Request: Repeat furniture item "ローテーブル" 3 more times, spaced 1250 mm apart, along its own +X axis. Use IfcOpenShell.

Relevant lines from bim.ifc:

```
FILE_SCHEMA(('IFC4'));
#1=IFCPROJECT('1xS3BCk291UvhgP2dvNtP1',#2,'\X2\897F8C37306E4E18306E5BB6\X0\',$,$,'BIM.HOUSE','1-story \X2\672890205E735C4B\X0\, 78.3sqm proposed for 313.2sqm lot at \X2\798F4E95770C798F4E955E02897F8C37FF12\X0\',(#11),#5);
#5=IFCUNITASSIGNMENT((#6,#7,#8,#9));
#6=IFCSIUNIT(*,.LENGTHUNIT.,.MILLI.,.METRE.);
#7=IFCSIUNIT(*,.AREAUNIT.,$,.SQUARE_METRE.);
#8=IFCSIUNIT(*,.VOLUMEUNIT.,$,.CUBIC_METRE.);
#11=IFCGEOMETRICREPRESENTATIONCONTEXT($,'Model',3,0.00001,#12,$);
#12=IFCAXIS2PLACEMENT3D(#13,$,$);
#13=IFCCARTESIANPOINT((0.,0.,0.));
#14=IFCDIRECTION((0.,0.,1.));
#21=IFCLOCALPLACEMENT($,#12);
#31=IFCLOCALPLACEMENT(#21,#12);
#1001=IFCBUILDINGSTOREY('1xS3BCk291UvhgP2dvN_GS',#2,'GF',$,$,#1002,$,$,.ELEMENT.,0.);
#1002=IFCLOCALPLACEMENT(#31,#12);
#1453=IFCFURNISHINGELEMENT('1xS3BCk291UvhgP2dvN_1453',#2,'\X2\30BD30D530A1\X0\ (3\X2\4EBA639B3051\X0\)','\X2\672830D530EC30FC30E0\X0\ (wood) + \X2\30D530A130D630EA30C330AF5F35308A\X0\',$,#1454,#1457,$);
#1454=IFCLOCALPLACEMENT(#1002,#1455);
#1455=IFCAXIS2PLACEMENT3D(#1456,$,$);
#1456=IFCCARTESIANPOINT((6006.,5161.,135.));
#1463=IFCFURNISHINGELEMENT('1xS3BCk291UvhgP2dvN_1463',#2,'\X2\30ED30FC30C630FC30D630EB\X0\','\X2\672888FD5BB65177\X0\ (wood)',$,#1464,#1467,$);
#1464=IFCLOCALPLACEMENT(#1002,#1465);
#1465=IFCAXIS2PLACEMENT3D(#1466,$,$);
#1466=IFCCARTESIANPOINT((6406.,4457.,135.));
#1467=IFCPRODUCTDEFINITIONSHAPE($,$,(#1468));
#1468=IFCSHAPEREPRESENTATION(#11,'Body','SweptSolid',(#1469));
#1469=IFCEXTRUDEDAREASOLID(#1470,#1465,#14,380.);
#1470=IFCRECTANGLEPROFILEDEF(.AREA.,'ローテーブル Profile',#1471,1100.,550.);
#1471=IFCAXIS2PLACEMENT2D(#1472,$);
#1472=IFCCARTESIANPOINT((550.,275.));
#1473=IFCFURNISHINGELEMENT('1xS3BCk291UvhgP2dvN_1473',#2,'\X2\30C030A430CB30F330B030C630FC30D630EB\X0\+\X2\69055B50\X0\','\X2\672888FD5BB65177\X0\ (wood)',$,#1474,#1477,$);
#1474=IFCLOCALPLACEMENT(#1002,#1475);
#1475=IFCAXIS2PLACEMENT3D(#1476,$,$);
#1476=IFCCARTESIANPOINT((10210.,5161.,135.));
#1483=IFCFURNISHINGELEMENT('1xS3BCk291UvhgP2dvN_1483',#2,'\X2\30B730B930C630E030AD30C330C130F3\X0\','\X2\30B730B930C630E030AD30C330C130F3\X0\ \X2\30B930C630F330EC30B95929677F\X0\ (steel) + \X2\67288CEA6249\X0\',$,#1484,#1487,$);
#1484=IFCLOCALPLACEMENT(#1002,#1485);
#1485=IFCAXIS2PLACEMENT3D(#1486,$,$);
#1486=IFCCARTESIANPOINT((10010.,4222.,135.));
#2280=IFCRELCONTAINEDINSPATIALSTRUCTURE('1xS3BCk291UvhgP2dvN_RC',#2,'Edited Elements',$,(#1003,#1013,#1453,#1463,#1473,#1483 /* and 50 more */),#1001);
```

```python
import ifcopenshell
import ifcopenshell.api.geometry
import ifcopenshell.api.root
import ifcopenshell.util.element
import ifcopenshell.util.placement
import ifcopenshell.util.unit

model = ifcopenshell.open("bim.ifc")
unit_scale = ifcopenshell.util.unit.calculate_unit_scale(model)


def reuse_history(source, copy):
    """copy_class also copies each property set's owner history, people and application; keep the originals."""
    for rel in copy.IsDefinedBy:
        if rel.is_a("IfcRelDefinesByProperties") and (history := rel.RelatingPropertyDefinition.OwnerHistory):
            rel.RelatingPropertyDefinition.OwnerHistory = source.OwnerHistory
            ifcopenshell.util.element.remove_deep2(model, history)


source = model.by_guid("1xS3BCk291UvhgP2dvN_1463")
base = ifcopenshell.util.placement.get_local_placement(source.ObjectPlacement)
step = base[:3, 0] * 1.25 / unit_scale

for i in range(1, 4):
    copy = ifcopenshell.api.root.copy_class(model, product=source)
    copy.Representation = ifcopenshell.util.element.copy_deep(
        model, source.Representation, exclude=["IfcGeometricRepresentationContext", "IfcRepresentationMap"]
    )
    reuse_history(source, copy)
    matrix = base.copy()
    matrix[:3, 3] += i * step
    print("added at", matrix[:3, 3].round(3) + 0.0)
    ifcopenshell.api.geometry.edit_object_placement(model, product=copy, matrix=matrix, is_si=False)

model.write("bim_edited.ifc")
```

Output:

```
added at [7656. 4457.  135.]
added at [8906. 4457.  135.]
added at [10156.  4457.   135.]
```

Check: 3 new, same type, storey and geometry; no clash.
